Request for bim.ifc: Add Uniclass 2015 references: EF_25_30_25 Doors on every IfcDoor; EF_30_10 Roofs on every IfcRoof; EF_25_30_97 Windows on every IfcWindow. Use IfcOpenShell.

First a look at what the model holds.

```python
import ifcopenshell

model = ifcopenshell.open("bim.ifc")
print(model.schema)
print("classifications:", [c.Name for c in model.by_type("IfcClassification")])
for ifc_class in ("IfcDoor", "IfcRoof", "IfcStair", "IfcWall", "IfcWindow"):
    print(ifc_class, len(model.by_type(ifc_class)))
```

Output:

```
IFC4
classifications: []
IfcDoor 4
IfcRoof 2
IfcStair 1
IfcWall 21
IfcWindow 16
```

```python
import ifcopenshell
import ifcopenshell.api.classification

model = ifcopenshell.open("bim.ifc")

system = ifcopenshell.api.classification.add_classification(model, classification="Uniclass 2015")

codes = {
    "IfcDoor": ("EF_25_30_25", "Doors"),
    "IfcRoof": ("EF_30_10", "Roofs"),
    "IfcWindow": ("EF_25_30_97", "Windows"),
}
for ifc_class, (code, name) in codes.items():
    products = model.by_type(ifc_class)
    ifcopenshell.api.classification.add_reference(
        model, products=products, classification=system, identification=code, name=name
    )
    print(code, len(products))

model.write("bim_v2.ifc")
```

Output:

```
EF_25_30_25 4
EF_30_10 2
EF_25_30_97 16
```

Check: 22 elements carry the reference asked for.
